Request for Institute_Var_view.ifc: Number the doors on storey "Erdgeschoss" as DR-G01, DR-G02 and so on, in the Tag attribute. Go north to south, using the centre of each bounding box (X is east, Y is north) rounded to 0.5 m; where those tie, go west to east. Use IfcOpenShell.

First a look at what the model holds.

```python
import ifcopenshell
import ifcopenshell.util.element
import ifcopenshell.util.placement

model = ifcopenshell.open("Institute_Var_view.ifc")
print(model.schema)
storey = next(s for s in model.by_type("IfcBuildingStorey") if s.Name == "Erdgeschoss")
doors = [e for e in ifcopenshell.util.element.get_decomposition(storey) if e.is_a("IfcDoor")]
for e in sorted(doors, key=lambda e: e.id()):
    origin = ifcopenshell.util.placement.get_local_placement(e.ObjectPlacement)[:3, 3]
    print(e.id(), e.Tag, e.Name, origin.round(2) + 0.0, sep=" | ")
```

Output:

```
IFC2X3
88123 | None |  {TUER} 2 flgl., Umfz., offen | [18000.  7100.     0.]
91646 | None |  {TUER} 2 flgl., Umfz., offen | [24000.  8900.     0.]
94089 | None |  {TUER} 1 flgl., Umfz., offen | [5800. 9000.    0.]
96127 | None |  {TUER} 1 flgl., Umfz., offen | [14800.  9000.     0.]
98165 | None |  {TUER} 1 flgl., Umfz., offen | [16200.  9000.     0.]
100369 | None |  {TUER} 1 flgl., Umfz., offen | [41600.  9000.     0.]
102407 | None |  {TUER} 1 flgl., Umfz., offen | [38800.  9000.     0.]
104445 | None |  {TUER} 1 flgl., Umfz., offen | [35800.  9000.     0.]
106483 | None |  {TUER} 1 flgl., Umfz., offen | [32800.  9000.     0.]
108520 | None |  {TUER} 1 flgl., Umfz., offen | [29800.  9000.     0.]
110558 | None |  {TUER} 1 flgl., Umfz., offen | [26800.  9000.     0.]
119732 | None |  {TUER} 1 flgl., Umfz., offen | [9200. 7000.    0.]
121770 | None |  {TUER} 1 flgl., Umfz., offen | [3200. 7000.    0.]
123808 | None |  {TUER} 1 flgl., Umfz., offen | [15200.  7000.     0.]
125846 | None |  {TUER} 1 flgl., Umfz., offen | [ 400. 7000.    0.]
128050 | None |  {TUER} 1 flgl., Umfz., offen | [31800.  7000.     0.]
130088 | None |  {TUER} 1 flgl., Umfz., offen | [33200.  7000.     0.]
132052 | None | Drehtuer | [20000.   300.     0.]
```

```python
import ifcopenshell
import ifcopenshell.geom
import ifcopenshell.util.element
import ifcopenshell.util.shape

model = ifcopenshell.open("Institute_Var_view.ifc")
settings = ifcopenshell.geom.settings()
settings.set("use-world-coords", True)


def centre(element):
    shape = ifcopenshell.geom.create_shape(settings, element)
    return ifcopenshell.util.shape.get_bbox_centroid(shape.geometry)


storey = next(s for s in model.by_type("IfcBuildingStorey") if s.Name == "Erdgeschoss")
doors = [e for e in ifcopenshell.util.element.get_decomposition(storey) if e.is_a("IfcDoor")]

# Insertion points can sit at a corner or the storey origin, so sort by the geometry (in metres).
centres = {e: centre(e) for e in doors}
doors.sort(key=lambda e: (-round(centres[e][1] / 0.5), centres[e][0]))

for i, e in enumerate(doors, start=1):
    number = f"DR-G{i:02d}"
    e.Tag = number
    print(e.id(), number)

model.write("Institute_Var_view_edited.ifc")
```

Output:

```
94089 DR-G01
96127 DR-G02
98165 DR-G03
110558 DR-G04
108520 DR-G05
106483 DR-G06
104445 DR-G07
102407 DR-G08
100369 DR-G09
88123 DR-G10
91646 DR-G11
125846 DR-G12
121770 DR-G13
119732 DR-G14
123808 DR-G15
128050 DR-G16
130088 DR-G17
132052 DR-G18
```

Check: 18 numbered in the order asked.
